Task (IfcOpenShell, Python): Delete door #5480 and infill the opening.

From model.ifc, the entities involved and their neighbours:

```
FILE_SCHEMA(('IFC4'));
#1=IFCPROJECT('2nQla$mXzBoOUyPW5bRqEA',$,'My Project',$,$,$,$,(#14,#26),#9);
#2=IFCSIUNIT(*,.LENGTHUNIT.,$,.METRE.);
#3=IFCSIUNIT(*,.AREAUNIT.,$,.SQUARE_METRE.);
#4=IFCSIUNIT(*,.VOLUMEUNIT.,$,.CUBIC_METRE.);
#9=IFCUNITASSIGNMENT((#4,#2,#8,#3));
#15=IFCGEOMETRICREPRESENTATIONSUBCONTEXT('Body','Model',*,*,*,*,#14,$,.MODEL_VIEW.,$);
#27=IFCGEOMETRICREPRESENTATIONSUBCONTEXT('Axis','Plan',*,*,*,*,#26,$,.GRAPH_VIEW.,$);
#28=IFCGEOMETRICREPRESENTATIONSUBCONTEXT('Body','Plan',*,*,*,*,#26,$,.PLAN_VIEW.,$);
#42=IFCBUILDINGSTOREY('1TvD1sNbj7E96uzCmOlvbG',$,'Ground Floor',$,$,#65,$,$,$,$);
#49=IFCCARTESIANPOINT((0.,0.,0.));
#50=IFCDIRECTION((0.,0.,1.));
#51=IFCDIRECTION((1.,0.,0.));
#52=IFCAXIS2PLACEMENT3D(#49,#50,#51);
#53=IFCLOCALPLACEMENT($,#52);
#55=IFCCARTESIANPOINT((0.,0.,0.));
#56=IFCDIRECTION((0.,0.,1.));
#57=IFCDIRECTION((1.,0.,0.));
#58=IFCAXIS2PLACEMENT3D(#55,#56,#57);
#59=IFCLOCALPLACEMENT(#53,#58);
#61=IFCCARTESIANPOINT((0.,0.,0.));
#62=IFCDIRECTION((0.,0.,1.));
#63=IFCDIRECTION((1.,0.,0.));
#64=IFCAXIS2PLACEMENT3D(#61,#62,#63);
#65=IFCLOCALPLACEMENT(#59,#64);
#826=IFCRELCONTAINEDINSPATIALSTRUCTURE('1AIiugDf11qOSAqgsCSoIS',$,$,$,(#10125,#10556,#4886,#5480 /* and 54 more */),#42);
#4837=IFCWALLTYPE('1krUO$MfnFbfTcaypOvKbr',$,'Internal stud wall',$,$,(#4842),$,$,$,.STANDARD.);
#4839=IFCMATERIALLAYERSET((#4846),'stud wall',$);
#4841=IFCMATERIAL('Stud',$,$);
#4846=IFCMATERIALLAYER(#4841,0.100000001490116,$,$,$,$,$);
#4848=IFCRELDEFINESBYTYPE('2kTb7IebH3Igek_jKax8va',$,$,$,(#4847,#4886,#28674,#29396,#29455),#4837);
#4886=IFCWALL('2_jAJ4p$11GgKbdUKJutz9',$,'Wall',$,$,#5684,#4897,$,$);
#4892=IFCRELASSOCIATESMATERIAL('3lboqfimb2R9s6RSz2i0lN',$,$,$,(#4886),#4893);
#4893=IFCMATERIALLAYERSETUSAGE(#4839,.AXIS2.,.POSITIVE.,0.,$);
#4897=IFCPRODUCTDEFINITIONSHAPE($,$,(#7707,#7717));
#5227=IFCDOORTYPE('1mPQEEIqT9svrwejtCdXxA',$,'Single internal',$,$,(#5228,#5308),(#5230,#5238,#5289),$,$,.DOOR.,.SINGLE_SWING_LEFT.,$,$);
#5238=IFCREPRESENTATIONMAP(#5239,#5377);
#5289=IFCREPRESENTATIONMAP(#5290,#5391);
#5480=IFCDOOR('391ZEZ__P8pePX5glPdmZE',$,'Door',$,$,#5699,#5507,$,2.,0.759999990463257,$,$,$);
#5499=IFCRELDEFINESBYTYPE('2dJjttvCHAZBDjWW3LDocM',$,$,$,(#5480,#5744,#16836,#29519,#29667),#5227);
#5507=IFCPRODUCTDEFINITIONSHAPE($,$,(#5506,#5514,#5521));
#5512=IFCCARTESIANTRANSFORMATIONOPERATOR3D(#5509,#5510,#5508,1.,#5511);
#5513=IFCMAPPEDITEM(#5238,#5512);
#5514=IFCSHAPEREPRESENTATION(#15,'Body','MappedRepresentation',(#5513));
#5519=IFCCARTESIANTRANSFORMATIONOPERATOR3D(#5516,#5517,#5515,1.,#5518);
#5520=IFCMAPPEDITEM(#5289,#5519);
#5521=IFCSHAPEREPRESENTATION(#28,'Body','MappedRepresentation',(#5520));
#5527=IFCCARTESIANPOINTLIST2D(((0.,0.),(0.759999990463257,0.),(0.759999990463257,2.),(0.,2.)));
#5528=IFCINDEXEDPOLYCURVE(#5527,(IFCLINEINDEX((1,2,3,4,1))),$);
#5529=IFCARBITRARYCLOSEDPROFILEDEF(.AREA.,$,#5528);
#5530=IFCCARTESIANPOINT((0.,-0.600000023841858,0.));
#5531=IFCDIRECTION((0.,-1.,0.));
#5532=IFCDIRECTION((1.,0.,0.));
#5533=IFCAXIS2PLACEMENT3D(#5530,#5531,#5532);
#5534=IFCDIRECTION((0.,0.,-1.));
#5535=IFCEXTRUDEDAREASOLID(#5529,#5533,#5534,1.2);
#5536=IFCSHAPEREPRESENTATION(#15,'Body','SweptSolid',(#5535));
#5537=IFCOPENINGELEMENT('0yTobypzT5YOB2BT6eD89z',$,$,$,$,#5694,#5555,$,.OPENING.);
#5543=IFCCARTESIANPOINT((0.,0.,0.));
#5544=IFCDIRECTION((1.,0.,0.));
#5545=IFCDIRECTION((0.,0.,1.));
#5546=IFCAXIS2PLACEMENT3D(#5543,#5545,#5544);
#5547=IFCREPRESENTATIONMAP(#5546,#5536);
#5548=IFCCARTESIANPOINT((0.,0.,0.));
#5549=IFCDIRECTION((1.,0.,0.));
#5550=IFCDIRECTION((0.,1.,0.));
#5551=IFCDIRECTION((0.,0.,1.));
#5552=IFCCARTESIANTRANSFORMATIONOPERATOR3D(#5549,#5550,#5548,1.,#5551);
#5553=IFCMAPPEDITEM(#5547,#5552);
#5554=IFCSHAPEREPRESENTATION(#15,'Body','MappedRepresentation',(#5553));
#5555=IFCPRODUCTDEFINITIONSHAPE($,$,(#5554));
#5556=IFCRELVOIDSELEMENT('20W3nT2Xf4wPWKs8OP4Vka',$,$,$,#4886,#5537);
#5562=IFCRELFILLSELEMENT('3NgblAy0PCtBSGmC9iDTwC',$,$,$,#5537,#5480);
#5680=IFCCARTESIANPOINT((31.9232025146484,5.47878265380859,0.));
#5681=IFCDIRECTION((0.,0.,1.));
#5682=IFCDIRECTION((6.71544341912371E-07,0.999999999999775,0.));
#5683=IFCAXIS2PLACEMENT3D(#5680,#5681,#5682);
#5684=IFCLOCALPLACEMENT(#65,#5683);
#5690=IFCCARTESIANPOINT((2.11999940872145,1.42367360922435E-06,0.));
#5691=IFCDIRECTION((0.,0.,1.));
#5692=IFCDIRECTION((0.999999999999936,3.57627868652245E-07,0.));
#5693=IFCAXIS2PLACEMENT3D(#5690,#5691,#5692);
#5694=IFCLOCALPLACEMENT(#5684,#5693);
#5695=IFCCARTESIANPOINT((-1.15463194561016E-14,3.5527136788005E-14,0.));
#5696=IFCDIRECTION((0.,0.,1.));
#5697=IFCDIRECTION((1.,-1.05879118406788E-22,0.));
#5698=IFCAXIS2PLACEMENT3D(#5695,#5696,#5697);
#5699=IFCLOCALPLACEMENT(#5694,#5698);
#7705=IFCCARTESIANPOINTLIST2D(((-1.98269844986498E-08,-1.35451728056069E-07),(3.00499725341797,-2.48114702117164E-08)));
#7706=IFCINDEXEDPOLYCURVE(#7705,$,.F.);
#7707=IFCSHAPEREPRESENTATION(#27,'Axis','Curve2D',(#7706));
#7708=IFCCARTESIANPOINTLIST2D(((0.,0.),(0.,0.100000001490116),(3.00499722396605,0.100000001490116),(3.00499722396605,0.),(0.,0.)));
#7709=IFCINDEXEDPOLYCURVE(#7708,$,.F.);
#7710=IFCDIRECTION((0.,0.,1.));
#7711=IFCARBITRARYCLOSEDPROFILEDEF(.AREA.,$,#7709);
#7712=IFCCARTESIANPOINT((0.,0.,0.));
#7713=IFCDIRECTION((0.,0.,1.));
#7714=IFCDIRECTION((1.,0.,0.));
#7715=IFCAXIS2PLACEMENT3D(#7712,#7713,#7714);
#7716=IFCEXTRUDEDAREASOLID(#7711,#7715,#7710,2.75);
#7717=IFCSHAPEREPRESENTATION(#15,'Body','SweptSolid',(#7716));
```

```python
import ifcopenshell
import ifcopenshell.api.feature
import ifcopenshell.api.root
import ifcopenshell.geom
import ifcopenshell.util.shape

model = ifcopenshell.open("model.ifc")
settings = ifcopenshell.geom.settings()


def volume(element):
    """Net volume in cubic metres, openings subtracted."""
    shape = ifcopenshell.geom.create_shape(settings, element)
    return ifcopenshell.util.shape.get_volume(shape.geometry)


door = model.by_id(5480)
opening = door.FillsVoids[0].RelatingOpeningElement
wall = opening.VoidsElements[0].RelatingBuildingElement
before = volume(wall)

ifcopenshell.api.root.remove_product(model, product=door)
ifcopenshell.api.feature.remove_feature(model, feature=opening)

after = volume(wall)

print(f"wall volume {before:.3f} -> {after:.3f} m3")

model.write("model_rev.ifc")
```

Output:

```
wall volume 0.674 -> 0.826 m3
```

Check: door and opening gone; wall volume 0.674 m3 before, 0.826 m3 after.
